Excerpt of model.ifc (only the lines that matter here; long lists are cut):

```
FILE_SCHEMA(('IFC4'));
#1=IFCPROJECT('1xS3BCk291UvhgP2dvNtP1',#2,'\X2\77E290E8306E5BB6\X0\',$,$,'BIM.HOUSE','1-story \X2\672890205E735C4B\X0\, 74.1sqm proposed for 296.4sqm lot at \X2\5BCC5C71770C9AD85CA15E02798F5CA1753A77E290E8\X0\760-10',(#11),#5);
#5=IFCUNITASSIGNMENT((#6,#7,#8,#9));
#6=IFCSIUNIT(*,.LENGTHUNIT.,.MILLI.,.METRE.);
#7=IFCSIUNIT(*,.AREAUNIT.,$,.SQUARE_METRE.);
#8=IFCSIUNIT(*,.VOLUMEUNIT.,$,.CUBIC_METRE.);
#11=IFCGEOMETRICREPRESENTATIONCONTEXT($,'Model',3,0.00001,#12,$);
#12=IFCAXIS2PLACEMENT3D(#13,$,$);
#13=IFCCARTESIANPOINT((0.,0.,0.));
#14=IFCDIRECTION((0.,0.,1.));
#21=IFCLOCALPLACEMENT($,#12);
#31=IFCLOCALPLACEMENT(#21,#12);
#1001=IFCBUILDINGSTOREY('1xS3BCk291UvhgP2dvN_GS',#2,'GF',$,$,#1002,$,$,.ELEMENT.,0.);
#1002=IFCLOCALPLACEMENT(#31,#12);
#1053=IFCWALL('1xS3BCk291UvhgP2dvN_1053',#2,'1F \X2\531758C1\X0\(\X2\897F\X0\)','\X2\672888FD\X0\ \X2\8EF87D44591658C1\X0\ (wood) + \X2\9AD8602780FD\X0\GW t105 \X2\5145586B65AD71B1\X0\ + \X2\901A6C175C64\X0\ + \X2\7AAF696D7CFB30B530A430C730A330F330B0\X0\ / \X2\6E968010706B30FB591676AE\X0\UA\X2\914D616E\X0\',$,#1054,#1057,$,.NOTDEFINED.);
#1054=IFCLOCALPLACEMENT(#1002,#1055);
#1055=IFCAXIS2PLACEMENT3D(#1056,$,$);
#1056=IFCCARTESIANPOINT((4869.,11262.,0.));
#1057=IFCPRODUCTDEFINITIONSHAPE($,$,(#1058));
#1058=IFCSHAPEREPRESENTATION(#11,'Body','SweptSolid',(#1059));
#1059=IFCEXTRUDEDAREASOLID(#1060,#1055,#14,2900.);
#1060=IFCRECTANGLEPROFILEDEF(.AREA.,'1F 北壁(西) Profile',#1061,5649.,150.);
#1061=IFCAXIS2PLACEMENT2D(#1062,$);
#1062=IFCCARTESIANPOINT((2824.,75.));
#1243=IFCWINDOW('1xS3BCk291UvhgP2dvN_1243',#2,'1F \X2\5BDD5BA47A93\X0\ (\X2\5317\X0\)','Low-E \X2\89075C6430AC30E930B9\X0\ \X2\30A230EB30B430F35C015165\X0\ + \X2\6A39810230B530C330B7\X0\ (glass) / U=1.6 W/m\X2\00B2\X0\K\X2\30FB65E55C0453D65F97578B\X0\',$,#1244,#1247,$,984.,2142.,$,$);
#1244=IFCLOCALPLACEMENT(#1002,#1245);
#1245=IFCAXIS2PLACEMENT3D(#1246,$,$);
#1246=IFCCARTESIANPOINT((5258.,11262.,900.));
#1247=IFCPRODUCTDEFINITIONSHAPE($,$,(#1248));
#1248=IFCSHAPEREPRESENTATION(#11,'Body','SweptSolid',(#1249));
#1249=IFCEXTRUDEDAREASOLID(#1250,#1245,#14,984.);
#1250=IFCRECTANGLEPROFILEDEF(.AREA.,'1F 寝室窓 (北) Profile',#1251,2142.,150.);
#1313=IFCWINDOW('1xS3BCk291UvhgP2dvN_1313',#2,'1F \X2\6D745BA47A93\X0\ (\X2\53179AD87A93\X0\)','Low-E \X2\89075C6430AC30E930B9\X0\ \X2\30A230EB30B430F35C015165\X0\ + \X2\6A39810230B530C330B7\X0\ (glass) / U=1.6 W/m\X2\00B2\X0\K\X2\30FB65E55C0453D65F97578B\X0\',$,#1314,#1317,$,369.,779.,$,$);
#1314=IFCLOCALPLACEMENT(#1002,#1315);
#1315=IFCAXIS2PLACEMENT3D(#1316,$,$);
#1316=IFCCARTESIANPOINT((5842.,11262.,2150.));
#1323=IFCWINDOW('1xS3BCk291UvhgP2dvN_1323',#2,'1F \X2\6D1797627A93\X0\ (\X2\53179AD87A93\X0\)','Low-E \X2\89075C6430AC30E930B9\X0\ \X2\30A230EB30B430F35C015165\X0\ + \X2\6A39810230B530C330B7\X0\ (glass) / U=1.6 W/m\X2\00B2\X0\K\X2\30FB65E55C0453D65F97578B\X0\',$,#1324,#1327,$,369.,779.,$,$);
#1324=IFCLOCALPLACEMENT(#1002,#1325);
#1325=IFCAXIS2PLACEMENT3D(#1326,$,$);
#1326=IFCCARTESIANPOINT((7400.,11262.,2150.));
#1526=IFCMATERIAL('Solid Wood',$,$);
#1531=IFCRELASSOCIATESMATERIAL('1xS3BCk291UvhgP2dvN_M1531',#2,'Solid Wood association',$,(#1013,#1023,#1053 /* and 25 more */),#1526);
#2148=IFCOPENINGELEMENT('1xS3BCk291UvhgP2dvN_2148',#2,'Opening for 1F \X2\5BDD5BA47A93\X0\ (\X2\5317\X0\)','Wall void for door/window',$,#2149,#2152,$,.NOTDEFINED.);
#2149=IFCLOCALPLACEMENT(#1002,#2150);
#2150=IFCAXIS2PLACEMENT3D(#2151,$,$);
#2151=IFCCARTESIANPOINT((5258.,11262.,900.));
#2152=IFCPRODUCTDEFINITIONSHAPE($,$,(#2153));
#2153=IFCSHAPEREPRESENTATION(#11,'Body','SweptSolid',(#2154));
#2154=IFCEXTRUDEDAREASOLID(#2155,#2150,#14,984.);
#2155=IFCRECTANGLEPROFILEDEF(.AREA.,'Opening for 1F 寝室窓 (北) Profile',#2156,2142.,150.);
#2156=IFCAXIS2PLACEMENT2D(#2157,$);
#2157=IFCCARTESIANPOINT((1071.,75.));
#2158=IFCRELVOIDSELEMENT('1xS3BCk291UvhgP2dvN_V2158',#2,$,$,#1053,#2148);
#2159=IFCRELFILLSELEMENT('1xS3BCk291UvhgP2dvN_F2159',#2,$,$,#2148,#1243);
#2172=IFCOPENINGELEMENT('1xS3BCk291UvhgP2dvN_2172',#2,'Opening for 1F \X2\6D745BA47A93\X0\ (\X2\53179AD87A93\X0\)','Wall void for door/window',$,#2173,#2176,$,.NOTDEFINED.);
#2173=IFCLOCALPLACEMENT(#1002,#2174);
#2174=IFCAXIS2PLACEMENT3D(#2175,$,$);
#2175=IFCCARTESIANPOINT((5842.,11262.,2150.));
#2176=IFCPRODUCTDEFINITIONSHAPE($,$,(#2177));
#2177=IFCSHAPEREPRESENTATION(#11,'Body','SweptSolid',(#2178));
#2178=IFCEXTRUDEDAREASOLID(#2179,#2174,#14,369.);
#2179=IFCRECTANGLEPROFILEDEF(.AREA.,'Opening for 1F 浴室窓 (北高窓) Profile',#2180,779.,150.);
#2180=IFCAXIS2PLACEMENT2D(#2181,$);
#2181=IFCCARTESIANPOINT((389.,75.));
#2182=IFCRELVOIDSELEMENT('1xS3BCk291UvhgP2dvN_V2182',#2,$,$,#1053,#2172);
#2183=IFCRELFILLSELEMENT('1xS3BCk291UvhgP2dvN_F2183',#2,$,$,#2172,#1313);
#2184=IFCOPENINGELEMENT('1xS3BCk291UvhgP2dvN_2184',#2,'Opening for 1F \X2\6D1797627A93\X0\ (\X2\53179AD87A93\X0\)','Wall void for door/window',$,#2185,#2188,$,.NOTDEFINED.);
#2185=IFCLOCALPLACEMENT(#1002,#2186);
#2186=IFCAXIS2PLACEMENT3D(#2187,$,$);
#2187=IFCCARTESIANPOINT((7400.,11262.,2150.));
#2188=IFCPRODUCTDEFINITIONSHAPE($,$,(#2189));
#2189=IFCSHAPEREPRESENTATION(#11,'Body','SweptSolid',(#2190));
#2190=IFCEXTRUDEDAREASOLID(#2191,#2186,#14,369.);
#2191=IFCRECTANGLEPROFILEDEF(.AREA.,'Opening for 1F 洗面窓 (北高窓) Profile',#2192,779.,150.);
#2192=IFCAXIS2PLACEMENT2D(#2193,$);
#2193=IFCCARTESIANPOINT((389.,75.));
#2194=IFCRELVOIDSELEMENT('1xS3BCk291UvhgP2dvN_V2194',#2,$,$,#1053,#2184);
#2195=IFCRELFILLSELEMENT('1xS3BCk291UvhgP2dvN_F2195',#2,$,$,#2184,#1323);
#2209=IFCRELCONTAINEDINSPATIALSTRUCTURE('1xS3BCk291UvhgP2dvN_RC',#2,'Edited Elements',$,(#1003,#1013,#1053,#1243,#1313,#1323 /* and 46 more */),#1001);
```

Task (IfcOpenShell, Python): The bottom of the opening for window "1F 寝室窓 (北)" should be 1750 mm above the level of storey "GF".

```python
import numpy as np
import ifcopenshell
import ifcopenshell.api.geometry
import ifcopenshell.geom
import ifcopenshell.util.element
import ifcopenshell.util.placement
import ifcopenshell.util.shape
import ifcopenshell.util.unit

model = ifcopenshell.open("model.ifc")
unit_scale = ifcopenshell.util.unit.calculate_unit_scale(model)

window = model.by_id(1243)
opening = window.FillsVoids[0].RelatingOpeningElement
storey = ifcopenshell.util.element.get_container(window, ifc_class="IfcBuildingStorey")
level = ifcopenshell.util.placement.get_local_placement(storey.ObjectPlacement)[2, 3]

# The opening's origin need not be at the sill, so measure its lowest point.
shape = ifcopenshell.geom.create_shape(ifcopenshell.geom.settings(), opening)
bottom = ifcopenshell.util.shape.get_shape_bottom_elevation(shape, shape.geometry) / unit_scale
dz = level + 1.75 / unit_scale - bottom

shift = np.array([0.0, 0.0, dz])
# The window is not placed relative to its opening, so move both.
for product in (opening, window):
    matrix = ifcopenshell.util.placement.get_local_placement(product.ObjectPlacement)
    matrix[:3, 3] += shift
    ifcopenshell.api.geometry.edit_object_placement(model, product=product, matrix=matrix, is_si=False)

print(f"moved by {dz * unit_scale:+.3f} m")

model.write("model-out.ifc")
```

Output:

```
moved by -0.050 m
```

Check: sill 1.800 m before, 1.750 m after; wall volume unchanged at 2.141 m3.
